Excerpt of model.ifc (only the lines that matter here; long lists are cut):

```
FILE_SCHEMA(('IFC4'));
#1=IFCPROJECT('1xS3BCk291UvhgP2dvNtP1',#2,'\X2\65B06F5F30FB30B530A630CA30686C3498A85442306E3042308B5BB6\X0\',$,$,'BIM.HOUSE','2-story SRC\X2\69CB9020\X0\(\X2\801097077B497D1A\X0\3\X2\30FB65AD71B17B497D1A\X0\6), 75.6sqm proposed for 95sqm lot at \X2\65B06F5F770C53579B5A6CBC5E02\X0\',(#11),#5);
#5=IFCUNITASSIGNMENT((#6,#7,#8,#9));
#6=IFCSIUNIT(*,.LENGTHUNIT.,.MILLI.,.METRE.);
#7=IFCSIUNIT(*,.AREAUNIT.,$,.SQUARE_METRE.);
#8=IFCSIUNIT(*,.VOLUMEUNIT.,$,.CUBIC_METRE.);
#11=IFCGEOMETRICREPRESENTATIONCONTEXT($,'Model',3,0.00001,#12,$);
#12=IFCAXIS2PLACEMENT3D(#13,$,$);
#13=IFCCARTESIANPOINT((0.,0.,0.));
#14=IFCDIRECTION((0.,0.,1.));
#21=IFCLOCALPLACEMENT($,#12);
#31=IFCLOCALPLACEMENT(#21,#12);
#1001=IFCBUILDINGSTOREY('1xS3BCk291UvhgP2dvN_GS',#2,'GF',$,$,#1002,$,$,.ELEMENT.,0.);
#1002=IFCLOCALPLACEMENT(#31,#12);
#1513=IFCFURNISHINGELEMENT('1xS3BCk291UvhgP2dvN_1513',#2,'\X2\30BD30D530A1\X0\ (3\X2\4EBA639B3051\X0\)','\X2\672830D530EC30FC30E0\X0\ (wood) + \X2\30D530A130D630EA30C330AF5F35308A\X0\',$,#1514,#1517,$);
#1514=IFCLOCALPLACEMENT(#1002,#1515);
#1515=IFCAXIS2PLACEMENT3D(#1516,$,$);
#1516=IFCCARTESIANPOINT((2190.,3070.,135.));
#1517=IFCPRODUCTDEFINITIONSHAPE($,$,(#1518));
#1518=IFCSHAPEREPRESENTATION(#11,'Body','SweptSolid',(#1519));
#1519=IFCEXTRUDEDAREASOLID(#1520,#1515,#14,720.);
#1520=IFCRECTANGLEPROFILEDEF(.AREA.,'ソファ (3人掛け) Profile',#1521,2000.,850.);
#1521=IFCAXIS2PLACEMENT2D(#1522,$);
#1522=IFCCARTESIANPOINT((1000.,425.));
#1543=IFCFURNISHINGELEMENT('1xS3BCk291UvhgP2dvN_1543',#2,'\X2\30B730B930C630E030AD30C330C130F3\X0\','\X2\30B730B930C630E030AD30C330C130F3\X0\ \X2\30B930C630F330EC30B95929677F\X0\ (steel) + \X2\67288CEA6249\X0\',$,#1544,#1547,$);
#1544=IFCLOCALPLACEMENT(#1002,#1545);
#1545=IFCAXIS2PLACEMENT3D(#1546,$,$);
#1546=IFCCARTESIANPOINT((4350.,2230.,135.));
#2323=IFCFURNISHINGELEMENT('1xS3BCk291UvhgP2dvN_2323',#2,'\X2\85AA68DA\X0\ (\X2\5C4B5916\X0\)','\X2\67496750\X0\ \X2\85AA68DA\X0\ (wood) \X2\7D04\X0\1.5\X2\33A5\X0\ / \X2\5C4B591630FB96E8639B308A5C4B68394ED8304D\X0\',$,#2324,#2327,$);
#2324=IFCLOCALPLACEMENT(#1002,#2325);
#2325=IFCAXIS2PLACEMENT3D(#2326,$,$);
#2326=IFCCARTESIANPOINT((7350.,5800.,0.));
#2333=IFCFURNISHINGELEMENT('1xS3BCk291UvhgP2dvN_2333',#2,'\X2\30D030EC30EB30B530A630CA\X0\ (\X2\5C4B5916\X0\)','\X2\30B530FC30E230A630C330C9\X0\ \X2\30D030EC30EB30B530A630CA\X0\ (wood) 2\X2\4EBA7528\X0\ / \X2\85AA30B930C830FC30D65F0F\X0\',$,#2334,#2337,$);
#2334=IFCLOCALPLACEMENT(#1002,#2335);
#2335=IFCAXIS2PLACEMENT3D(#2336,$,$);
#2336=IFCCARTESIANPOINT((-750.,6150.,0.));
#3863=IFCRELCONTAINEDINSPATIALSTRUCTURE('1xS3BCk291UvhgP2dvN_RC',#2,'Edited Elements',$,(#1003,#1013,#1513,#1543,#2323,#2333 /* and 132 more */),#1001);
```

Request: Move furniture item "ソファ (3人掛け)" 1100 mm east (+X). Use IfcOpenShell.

```python
import ifcopenshell
import ifcopenshell.api.geometry
import ifcopenshell.util.placement

model = ifcopenshell.open("model.ifc")

item = model.by_guid("1xS3BCk291UvhgP2dvN_1513")
matrix = ifcopenshell.util.placement.get_local_placement(item.ObjectPlacement)
matrix[0, 3] += 1100.0
ifcopenshell.api.geometry.edit_object_placement(model, product=item, matrix=matrix, is_si=False)

print(ifcopenshell.util.placement.get_local_placement(item.ObjectPlacement).round(3) + 0.0)

model.write("model_v2.ifc")
```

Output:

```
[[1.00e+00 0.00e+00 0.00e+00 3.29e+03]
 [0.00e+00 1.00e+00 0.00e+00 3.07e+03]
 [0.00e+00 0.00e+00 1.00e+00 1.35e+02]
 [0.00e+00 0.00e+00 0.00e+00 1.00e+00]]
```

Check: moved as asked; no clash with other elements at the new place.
